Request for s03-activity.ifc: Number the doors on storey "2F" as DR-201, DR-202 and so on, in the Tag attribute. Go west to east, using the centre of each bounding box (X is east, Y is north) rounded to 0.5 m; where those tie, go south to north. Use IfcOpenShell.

First a look at what the model holds.

```python
import ifcopenshell
import ifcopenshell.util.element
import ifcopenshell.util.placement

model = ifcopenshell.open("s03-activity.ifc")
print(model.schema)
storey = next(s for s in model.by_type("IfcBuildingStorey") if s.Name == "2F")
doors = [e for e in ifcopenshell.util.element.get_decomposition(storey) if e.is_a("IfcDoor")]
for e in sorted(doors, key=lambda e: e.id()):
    origin = ifcopenshell.util.placement.get_local_placement(e.ObjectPlacement)[:3, 3]
    print(e.id(), e.Tag, e.Name, origin.round(2) + 0.0, sep=" | ")
```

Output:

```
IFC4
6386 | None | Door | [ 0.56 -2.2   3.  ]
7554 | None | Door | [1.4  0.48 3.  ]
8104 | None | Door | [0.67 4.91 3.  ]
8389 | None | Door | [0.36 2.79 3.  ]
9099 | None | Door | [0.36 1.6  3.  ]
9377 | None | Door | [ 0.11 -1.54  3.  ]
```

```python
import ifcopenshell
import ifcopenshell.geom
import ifcopenshell.util.element
import ifcopenshell.util.shape

model = ifcopenshell.open("s03-activity.ifc")
settings = ifcopenshell.geom.settings()
settings.set("use-world-coords", True)


def centre(element):
    shape = ifcopenshell.geom.create_shape(settings, element)
    return ifcopenshell.util.shape.get_bbox_centroid(shape.geometry)


storey = next(s for s in model.by_type("IfcBuildingStorey") if s.Name == "2F")
doors = [e for e in ifcopenshell.util.element.get_decomposition(storey) if e.is_a("IfcDoor")]

# Insertion points can sit at a corner or the storey origin, so sort by the geometry (in metres).
centres = {e: centre(e) for e in doors}
doors.sort(key=lambda e: (round(centres[e][0] / 0.5), centres[e][1]))

for i, e in enumerate(doors, start=1):
    number = f"DR-2{i:02d}"
    e.Tag = number
    print(e.id(), number)

model.write("s03-activity_rev.ifc")
```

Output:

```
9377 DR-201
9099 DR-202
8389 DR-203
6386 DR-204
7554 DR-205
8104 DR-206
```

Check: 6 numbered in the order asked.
